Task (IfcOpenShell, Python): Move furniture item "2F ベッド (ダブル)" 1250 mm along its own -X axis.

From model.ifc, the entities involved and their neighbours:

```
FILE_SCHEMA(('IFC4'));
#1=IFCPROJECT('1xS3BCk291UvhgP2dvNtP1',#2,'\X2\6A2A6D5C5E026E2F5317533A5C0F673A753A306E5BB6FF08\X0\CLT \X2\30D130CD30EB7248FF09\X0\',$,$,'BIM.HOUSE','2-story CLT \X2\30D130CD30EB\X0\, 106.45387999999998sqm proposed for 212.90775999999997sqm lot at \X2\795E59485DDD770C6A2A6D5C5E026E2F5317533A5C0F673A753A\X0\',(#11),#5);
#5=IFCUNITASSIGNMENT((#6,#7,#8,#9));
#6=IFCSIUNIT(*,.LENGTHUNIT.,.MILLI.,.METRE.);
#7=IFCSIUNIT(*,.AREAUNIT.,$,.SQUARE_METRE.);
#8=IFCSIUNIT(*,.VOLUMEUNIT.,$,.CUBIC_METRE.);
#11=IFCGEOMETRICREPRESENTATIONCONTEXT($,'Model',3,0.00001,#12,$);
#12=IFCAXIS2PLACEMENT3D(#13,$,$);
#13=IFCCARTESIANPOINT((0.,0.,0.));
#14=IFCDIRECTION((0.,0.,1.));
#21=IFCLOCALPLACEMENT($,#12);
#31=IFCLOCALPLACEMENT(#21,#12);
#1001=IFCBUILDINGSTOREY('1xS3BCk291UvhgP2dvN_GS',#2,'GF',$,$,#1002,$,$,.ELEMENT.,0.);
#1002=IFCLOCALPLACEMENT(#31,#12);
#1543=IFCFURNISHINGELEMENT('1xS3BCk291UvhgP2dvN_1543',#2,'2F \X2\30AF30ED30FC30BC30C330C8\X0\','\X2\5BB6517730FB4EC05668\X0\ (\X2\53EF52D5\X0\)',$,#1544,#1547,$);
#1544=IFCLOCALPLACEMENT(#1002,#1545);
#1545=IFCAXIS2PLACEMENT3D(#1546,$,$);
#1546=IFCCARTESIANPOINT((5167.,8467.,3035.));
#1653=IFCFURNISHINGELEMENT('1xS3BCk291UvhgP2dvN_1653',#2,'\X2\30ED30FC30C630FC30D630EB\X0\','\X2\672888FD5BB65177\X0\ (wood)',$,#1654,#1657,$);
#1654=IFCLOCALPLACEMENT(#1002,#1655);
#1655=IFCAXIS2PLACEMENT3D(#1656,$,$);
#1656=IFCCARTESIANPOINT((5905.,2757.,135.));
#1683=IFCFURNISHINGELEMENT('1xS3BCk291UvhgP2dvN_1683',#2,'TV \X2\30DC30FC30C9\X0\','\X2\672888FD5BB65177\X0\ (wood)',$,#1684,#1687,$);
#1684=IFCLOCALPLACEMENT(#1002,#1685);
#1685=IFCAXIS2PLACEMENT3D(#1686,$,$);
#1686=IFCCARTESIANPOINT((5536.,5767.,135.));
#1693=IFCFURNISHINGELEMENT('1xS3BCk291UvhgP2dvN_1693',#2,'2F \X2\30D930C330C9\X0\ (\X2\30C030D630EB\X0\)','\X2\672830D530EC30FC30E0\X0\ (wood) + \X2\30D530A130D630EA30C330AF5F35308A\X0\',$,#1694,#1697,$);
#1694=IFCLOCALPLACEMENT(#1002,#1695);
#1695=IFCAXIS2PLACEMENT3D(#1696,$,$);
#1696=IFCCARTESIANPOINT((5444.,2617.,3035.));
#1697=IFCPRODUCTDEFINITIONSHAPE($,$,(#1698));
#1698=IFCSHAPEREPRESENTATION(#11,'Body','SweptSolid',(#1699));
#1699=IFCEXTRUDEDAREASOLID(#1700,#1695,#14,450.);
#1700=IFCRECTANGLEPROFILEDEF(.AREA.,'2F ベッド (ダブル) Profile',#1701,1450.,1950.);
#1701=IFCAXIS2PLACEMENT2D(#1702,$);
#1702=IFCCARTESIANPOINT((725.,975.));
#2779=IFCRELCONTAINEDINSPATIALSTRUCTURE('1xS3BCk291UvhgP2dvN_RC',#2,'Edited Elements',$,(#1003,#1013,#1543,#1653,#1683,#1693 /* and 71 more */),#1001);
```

```python
import ifcopenshell
import ifcopenshell.api.geometry
import ifcopenshell.util.placement
import ifcopenshell.util.unit

model = ifcopenshell.open("model.ifc")
unit_scale = ifcopenshell.util.unit.calculate_unit_scale(model)

item = model.by_guid("1xS3BCk291UvhgP2dvN_1693")
matrix = ifcopenshell.util.placement.get_local_placement(item.ObjectPlacement)
matrix[:3, 3] -= matrix[:3, 0] * 1.25 / unit_scale
ifcopenshell.api.geometry.edit_object_placement(model, product=item, matrix=matrix, is_si=False)

print(ifcopenshell.util.placement.get_local_placement(item.ObjectPlacement).round(3) + 0.0)

model.write("model-out.ifc")
```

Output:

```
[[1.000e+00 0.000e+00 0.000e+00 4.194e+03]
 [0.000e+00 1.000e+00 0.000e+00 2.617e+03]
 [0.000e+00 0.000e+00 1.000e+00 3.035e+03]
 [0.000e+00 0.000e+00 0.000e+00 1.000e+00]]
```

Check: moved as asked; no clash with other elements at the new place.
